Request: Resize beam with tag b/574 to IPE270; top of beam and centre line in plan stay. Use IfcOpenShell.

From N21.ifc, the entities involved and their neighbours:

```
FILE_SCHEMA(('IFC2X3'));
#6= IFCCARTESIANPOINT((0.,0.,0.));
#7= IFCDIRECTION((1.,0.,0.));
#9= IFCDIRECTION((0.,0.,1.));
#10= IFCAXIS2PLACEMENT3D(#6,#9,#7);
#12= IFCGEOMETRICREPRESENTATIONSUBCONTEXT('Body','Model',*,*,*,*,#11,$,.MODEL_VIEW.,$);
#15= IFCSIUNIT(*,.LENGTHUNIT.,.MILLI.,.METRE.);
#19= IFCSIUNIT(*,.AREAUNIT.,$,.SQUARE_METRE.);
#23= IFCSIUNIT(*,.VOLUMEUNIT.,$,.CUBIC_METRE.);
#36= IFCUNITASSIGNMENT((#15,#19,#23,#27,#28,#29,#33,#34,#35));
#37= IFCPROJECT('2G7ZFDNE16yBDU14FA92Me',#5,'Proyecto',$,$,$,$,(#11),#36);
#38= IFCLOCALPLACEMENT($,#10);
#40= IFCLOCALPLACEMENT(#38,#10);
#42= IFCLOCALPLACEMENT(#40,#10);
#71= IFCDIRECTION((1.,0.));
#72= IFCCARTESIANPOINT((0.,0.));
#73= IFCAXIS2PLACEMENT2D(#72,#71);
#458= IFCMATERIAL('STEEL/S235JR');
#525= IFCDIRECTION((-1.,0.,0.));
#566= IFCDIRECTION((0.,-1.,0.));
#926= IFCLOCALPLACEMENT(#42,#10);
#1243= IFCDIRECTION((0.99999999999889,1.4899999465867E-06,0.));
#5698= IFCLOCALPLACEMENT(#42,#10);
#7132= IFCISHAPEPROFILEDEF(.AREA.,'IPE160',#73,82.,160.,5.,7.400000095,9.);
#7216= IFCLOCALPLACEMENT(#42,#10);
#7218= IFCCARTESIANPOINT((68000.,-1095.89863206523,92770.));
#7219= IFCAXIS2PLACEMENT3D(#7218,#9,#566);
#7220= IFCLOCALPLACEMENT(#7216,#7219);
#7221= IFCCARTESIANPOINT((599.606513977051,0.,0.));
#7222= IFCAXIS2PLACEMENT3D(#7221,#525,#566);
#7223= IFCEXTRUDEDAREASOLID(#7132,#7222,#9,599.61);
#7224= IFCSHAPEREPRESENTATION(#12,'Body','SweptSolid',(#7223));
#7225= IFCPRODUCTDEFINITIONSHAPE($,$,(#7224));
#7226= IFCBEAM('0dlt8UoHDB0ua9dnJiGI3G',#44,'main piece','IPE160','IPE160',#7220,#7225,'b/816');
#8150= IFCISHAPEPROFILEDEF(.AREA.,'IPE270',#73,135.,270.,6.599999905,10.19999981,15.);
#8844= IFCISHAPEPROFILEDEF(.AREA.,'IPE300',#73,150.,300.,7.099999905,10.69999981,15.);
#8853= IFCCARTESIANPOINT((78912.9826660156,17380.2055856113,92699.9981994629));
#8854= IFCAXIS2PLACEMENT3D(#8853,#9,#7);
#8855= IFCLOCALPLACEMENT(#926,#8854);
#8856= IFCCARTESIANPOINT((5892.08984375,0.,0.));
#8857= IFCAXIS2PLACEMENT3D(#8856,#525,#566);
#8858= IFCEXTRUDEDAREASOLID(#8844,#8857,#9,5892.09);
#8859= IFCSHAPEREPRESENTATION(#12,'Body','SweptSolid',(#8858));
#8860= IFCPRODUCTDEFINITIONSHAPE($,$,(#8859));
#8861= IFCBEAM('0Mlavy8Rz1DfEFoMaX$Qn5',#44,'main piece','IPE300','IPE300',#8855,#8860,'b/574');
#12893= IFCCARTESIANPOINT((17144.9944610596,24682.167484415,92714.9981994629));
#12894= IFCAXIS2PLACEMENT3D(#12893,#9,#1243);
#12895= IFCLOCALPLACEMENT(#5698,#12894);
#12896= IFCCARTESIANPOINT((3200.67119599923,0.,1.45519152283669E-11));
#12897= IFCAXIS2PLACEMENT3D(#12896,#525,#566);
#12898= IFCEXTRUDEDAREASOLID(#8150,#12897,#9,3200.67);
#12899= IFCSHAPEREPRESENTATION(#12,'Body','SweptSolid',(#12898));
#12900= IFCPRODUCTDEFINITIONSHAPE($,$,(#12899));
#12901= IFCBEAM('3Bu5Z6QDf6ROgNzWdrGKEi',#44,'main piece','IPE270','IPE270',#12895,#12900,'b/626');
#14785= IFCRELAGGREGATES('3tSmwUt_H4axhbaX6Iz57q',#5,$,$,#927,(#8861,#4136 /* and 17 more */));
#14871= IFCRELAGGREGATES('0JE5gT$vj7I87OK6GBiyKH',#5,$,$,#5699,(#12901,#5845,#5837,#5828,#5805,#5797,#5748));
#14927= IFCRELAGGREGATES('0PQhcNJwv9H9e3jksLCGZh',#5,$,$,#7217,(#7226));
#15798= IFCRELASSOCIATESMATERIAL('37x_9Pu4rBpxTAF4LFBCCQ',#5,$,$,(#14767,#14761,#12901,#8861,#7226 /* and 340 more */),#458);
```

```python
import ifcopenshell
import ifcopenshell.util.element
import ifcopenshell.util.representation

model = ifcopenshell.open("N21.ifc")

member = model.by_id(8861)
source = next(p for p in model.by_type("IfcIShapeProfileDef") if p.ProfileName == "IPE270")

body = ifcopenshell.util.representation.get_representation(member, "Model", "Body")
solid = body.Items[0]
old_profile = solid.SweptArea

# Copy the section's sizes but keep this member's own profile position.
profile = ifcopenshell.util.element.copy(model, source)
# Profiles are centred, so shift by half the change in depth to hold the top.
shift = (old_profile.OverallDepth - profile.OverallDepth) / 2
x, y = old_profile.Position.Location.Coordinates
up = (0.0, 1.0)  # upwards, in the solid's own plane
location = model.createIfcCartesianPoint((x + up[0] * shift, y + up[1] * shift))
profile.Position = model.createIfcAxis2Placement2D(location, old_profile.Position.RefDirection)
solid.SweptArea = profile
if not model.get_total_inverses(old_profile):
    ifcopenshell.util.element.remove_deep2(model, old_profile)
member.Description = member.Description.replace("IPE300", "IPE270")
member.ObjectType = member.ObjectType.replace("IPE300", "IPE270")

print(solid.SweptArea)

model.write("N21-out.ifc")
```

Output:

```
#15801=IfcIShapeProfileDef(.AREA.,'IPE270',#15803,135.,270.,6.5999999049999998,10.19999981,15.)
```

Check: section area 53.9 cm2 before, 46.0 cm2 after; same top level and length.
